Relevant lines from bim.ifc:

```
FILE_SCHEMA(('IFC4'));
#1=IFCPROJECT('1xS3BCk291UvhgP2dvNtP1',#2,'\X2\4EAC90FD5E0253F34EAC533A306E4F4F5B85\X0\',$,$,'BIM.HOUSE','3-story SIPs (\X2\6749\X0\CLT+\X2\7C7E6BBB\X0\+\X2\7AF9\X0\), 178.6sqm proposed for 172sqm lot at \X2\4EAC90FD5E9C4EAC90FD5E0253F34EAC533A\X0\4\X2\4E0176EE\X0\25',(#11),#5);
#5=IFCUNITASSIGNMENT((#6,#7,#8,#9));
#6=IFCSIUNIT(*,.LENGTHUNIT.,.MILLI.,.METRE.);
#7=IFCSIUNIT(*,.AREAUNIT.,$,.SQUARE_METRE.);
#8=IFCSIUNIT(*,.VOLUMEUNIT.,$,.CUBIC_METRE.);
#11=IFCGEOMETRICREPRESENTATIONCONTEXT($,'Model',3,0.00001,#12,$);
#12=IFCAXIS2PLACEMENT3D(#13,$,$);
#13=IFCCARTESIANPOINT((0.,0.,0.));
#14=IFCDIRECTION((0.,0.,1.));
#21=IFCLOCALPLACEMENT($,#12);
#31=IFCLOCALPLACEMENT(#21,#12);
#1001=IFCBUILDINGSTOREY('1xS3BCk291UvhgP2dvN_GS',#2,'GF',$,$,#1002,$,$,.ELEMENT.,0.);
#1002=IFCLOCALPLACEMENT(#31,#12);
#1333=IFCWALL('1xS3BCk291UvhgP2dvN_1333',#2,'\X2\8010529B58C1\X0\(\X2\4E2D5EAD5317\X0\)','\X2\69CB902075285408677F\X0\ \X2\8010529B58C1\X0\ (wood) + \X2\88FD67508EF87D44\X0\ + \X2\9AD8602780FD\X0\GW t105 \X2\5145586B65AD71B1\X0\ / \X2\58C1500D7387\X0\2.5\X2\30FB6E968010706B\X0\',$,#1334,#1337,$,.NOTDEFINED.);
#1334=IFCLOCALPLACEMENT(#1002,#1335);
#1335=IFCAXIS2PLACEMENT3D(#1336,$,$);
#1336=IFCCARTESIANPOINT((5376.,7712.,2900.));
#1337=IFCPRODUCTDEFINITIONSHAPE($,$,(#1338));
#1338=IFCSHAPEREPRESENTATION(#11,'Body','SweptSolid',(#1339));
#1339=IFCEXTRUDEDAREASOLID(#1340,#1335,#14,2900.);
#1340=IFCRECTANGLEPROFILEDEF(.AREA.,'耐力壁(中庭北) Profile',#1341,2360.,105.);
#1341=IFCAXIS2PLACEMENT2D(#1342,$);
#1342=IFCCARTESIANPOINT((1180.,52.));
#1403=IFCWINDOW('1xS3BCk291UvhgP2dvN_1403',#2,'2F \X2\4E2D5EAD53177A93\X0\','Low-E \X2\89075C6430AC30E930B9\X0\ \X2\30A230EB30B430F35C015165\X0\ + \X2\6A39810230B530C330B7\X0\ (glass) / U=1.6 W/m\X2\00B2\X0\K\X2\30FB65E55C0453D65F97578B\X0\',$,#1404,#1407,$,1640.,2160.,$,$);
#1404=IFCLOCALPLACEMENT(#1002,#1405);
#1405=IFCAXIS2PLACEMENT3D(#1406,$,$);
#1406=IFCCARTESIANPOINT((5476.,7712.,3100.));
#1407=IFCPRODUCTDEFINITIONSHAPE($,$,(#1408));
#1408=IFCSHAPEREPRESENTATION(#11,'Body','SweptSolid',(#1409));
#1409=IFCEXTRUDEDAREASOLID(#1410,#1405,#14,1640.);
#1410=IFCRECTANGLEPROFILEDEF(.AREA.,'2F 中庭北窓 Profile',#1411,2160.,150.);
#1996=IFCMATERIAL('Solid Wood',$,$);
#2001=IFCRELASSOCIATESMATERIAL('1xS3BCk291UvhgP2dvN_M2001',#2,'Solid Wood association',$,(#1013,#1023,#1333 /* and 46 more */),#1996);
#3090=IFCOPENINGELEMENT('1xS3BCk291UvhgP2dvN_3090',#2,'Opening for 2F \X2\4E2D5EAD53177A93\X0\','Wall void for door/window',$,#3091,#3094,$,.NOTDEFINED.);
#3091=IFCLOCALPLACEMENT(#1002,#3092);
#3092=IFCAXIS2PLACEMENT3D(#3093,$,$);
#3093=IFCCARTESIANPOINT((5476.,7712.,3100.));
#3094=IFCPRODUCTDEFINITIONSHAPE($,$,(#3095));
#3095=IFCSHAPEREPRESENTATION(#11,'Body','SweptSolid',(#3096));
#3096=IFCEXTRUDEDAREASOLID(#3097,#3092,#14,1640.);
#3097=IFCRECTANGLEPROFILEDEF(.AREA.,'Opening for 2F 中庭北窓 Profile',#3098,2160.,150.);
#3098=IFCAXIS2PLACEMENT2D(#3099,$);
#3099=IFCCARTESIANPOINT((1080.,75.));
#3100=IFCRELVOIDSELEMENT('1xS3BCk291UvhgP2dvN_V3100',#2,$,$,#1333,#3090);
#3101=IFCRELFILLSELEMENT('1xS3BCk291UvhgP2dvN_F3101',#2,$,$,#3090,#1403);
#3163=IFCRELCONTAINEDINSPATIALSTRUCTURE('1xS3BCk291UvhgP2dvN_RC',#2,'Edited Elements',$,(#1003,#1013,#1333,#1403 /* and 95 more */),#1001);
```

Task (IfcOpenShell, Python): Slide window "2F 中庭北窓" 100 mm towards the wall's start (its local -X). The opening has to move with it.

```python
import ifcopenshell
import ifcopenshell.api.geometry
import ifcopenshell.util.placement

model = ifcopenshell.open("bim.ifc")

window = model.by_guid("1xS3BCk291UvhgP2dvN_1403")
opening = window.FillsVoids[0].RelatingOpeningElement
wall = opening.VoidsElements[0].RelatingBuildingElement

wall_matrix = ifcopenshell.util.placement.get_local_placement(wall.ObjectPlacement)
shift = wall_matrix[:3, 0] * -100.0
before = ifcopenshell.util.placement.get_local_placement(window.ObjectPlacement)[:3, 3].copy()

# The window is not placed relative to its opening, so move both.
for product in (opening, window):
    matrix = ifcopenshell.util.placement.get_local_placement(product.ObjectPlacement)
    matrix[:3, 3] += shift
    ifcopenshell.api.geometry.edit_object_placement(model, product=product, matrix=matrix, is_si=False)

after = ifcopenshell.util.placement.get_local_placement(window.ObjectPlacement)[:3, 3]
print("window moved by", (after - before).round(3) + 0.0)

model.write("bim_v2.ifc")
```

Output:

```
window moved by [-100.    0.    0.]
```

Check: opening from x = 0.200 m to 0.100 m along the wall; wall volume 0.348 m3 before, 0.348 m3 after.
